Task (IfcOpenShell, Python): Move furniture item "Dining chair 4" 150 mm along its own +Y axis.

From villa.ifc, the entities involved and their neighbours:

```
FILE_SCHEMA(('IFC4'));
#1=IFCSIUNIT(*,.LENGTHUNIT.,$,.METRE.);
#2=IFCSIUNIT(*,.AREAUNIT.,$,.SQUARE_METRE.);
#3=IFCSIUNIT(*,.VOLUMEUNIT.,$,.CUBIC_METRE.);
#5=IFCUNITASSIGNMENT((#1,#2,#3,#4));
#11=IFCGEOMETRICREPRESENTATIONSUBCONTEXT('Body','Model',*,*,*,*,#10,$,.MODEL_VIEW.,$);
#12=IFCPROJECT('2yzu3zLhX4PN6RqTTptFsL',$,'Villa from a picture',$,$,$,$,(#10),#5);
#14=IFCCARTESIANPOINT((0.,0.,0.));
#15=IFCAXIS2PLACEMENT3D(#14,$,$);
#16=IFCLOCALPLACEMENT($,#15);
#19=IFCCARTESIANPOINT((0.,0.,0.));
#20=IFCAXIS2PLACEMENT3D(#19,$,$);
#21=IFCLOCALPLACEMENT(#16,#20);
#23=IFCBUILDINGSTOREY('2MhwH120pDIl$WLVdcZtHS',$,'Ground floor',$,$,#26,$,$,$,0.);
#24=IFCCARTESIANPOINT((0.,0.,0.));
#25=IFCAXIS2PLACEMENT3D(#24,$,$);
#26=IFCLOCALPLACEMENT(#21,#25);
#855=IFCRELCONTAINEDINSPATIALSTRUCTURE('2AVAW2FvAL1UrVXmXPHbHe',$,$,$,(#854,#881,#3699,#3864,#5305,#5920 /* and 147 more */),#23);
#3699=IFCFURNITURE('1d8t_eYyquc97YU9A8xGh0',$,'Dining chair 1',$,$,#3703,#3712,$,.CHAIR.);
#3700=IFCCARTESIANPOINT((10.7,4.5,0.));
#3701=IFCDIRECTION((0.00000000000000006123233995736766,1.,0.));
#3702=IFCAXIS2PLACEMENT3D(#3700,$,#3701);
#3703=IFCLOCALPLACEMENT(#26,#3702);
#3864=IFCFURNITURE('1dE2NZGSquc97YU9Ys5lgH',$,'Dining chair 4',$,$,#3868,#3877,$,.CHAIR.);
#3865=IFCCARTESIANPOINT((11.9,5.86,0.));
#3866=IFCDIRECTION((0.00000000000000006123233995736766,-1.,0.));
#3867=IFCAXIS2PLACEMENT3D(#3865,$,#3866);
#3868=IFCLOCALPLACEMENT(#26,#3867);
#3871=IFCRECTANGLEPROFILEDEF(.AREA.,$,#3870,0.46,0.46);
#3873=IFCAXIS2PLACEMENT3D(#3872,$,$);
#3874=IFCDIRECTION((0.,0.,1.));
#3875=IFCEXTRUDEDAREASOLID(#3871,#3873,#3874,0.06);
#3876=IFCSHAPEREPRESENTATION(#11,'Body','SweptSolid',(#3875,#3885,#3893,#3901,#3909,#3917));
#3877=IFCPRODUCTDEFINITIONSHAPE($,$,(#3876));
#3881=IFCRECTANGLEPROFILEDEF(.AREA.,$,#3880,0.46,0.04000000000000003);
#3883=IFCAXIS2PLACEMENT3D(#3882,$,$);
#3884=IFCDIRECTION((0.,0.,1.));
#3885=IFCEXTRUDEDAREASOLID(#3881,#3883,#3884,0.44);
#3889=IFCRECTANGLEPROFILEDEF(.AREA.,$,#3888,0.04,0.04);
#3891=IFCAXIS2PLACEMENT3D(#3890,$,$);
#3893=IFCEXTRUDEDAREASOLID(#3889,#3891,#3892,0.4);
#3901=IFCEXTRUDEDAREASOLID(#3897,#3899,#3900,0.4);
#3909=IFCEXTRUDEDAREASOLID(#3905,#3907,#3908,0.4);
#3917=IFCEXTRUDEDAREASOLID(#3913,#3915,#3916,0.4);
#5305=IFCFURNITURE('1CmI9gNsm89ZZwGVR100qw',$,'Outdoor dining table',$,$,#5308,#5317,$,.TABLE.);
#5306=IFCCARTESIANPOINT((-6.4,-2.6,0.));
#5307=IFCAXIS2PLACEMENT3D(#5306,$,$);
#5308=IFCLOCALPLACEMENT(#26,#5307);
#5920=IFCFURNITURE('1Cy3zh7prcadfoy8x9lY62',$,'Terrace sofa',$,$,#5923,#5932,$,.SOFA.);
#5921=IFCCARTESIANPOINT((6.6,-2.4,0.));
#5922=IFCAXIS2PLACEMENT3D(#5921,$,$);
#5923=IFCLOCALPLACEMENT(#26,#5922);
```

```python
import ifcopenshell
import ifcopenshell.api.geometry
import ifcopenshell.util.placement
import ifcopenshell.util.unit

model = ifcopenshell.open("villa.ifc")
unit_scale = ifcopenshell.util.unit.calculate_unit_scale(model)

item = model.by_guid("1dE2NZGSquc97YU9Ys5lgH")
matrix = ifcopenshell.util.placement.get_local_placement(item.ObjectPlacement)
matrix[:3, 3] += matrix[:3, 1] * 0.15 / unit_scale
ifcopenshell.api.geometry.edit_object_placement(model, product=item, matrix=matrix, is_si=False)

print(ifcopenshell.util.placement.get_local_placement(item.ObjectPlacement).round(3) + 0.0)

model.write("villa_v2.ifc")
```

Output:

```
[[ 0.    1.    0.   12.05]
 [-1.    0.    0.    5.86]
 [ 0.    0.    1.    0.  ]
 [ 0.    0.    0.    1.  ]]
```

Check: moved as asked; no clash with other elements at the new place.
